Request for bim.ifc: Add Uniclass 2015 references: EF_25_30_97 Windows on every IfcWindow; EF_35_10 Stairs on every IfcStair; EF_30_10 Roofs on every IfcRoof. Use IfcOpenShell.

First a look at what the model holds.

```python
import ifcopenshell

model = ifcopenshell.open("bim.ifc")
print(model.schema)
print("classifications:", [c.Name for c in model.by_type("IfcClassification")])
for ifc_class in ("IfcDoor", "IfcRoof", "IfcStair", "IfcWall", "IfcWindow"):
    print(ifc_class, len(model.by_type(ifc_class)))
```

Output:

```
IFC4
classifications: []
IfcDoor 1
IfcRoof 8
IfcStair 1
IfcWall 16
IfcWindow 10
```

```python
import ifcopenshell
import ifcopenshell.api.classification

model = ifcopenshell.open("bim.ifc")

system = ifcopenshell.api.classification.add_classification(model, classification="Uniclass 2015")

codes = {
    "IfcWindow": ("EF_25_30_97", "Windows"),
    "IfcStair": ("EF_35_10", "Stairs"),
    "IfcRoof": ("EF_30_10", "Roofs"),
}
for ifc_class, (code, name) in codes.items():
    products = model.by_type(ifc_class)
    ifcopenshell.api.classification.add_reference(
        model, products=products, classification=system, identification=code, name=name
    )
    print(code, len(products))

model.write("bim-out.ifc")
```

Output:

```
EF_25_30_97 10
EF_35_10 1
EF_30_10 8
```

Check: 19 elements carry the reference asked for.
